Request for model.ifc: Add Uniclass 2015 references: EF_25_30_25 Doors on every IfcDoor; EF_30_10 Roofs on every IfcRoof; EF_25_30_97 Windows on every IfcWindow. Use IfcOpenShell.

First a look at what the model holds.

```python
import ifcopenshell

model = ifcopenshell.open("model.ifc")
print(model.schema)
print("classifications:", [c.Name for c in model.by_type("IfcClassification")])
for ifc_class in ("IfcDoor", "IfcRoof", "IfcStair", "IfcWall", "IfcWindow"):
    print(ifc_class, len(model.by_type(ifc_class)))
```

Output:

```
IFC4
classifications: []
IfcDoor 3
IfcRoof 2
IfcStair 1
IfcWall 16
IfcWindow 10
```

```python
import ifcopenshell
import ifcopenshell.api.classification

model = ifcopenshell.open("model.ifc")

system = ifcopenshell.api.classification.add_classification(model, classification="Uniclass 2015")

codes = {
    "IfcDoor": ("EF_25_30_25", "Doors"),
    "IfcRoof": ("EF_30_10", "Roofs"),
    "IfcWindow": ("EF_25_30_97", "Windows"),
}
for ifc_class, (code, name) in codes.items():
    products = model.by_type(ifc_class)
    ifcopenshell.api.classification.add_reference(
        model, products=products, classification=system, identification=code, name=name
    )
    print(code, len(products))

model.write("model_rev.ifc")
```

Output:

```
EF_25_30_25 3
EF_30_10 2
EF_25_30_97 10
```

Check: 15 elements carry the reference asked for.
